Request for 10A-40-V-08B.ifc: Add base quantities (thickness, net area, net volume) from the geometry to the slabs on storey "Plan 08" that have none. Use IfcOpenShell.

First a look at what the model holds.

```python
import ifcopenshell
import ifcopenshell.util.element
import ifcopenshell.util.unit

model = ifcopenshell.open("10A-40-V-08B.ifc")
print(model.schema)
for unit_type in ("LENGTHUNIT", "AREAUNIT", "VOLUMEUNIT"):
    print(unit_type, ifcopenshell.util.unit.calculate_unit_scale(model, unit_type))
storey = next(s for s in model.by_type("IfcBuildingStorey") if s.Name == "Plan 08")
slabs = [e for e in ifcopenshell.util.element.get_decomposition(storey) if e.is_a("IfcSlab")]
for e in sorted(slabs, key=lambda e: e.id()):
    print(e.id(), e.is_a(), e.Name, list(ifcopenshell.util.element.get_psets(e, qtos_only=True)), sep=" | ")
```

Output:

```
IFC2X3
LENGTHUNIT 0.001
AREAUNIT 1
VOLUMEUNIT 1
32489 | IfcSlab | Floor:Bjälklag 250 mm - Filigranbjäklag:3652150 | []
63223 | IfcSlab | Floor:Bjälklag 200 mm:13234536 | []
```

```python
import ifcopenshell
import ifcopenshell.api.pset
import ifcopenshell.geom
import ifcopenshell.util.element
import ifcopenshell.util.shape
import ifcopenshell.util.unit

model = ifcopenshell.open("10A-40-V-08B.ifc")
unit_scale = ifcopenshell.util.unit.calculate_unit_scale(model)
area_scale = ifcopenshell.util.unit.calculate_unit_scale(model, "AREAUNIT")
volume_scale = ifcopenshell.util.unit.calculate_unit_scale(model, "VOLUMEUNIT")
settings = ifcopenshell.geom.settings()

storey = next(s for s in model.by_type("IfcBuildingStorey") if s.Name == "Plan 08")
slabs = [e for e in ifcopenshell.util.element.get_decomposition(storey) if e.is_a("IfcSlab")]

for e in sorted(slabs, key=lambda e: e.id()):
    if ifcopenshell.util.element.get_psets(e, qtos_only=True, should_inherit=False):
        continue
    # Geometry comes back in metres, in the element's own axes.
    shape = ifcopenshell.geom.create_shape(settings, e)
    values = {
        "Width": ifcopenshell.util.shape.get_z(shape.geometry) / unit_scale,
        "NetArea": ifcopenshell.util.shape.get_footprint_area(shape.geometry) / area_scale,
        "NetVolume": ifcopenshell.util.shape.get_volume(shape.geometry) / volume_scale,
    }
    qto = ifcopenshell.api.pset.add_qto(model, product=e, name="BaseQuantities")
    ifcopenshell.api.pset.edit_qto(model, qto=qto, properties=values)
    print(e.id(), {k: round(v, 3) for k, v in values.items()})

model.write("10A-40-V-08B_v2.ifc")
```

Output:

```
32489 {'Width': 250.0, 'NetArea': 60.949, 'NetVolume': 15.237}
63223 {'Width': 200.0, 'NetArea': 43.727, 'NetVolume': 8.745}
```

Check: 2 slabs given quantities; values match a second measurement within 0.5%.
